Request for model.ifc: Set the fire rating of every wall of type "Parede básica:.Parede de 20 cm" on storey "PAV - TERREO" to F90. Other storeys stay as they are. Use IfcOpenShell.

First a look at what the model holds.

```python
import ifcopenshell
import ifcopenshell.util.element

model = ifcopenshell.open("model.ifc")
print(model.schema)
storey = next(s for s in model.by_type("IfcBuildingStorey") if s.Name == "PAV - TERREO")
walls = [e for e in ifcopenshell.util.element.get_decomposition(storey) if e.is_a("IfcWall")]
seen = {}
for e in walls:
    element_type = ifcopenshell.util.element.get_type(e)
    key = (element_type.Name if element_type != e and element_type else None, ifcopenshell.util.element.get_pset(e, "Pset_WallCommon", "FireRating"))
    seen[key] = seen.get(key, 0) + 1
for (name, value), count in sorted(seen.items(), key=str):
    print(count, "x", name, "|", value)
```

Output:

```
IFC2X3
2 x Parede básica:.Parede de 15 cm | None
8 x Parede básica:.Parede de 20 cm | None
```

```python
import ifcopenshell
import ifcopenshell.api.pset
import ifcopenshell.util.element

model = ifcopenshell.open("model.ifc")

storey = next(s for s in model.by_type("IfcBuildingStorey") if s.Name == "PAV - TERREO")
walls = [e for e in ifcopenshell.util.element.get_decomposition(storey) if e.is_a("IfcWall")]

count = 0
for e in walls:
    element_type = ifcopenshell.util.element.get_type(e)
    if element_type in (None, e) or element_type.Name != "Parede básica:.Parede de 20 cm":
        continue
    # add_pset returns the element's existing set when there is one.
    pset = ifcopenshell.api.pset.add_pset(model, product=e, name="Pset_WallCommon")
    ifcopenshell.api.pset.edit_pset(model, pset=pset, properties={"FireRating": "F90"})
    count += 1

print(count, "walls updated")

model.write("model_updated.ifc")
```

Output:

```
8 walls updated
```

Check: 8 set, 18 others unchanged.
